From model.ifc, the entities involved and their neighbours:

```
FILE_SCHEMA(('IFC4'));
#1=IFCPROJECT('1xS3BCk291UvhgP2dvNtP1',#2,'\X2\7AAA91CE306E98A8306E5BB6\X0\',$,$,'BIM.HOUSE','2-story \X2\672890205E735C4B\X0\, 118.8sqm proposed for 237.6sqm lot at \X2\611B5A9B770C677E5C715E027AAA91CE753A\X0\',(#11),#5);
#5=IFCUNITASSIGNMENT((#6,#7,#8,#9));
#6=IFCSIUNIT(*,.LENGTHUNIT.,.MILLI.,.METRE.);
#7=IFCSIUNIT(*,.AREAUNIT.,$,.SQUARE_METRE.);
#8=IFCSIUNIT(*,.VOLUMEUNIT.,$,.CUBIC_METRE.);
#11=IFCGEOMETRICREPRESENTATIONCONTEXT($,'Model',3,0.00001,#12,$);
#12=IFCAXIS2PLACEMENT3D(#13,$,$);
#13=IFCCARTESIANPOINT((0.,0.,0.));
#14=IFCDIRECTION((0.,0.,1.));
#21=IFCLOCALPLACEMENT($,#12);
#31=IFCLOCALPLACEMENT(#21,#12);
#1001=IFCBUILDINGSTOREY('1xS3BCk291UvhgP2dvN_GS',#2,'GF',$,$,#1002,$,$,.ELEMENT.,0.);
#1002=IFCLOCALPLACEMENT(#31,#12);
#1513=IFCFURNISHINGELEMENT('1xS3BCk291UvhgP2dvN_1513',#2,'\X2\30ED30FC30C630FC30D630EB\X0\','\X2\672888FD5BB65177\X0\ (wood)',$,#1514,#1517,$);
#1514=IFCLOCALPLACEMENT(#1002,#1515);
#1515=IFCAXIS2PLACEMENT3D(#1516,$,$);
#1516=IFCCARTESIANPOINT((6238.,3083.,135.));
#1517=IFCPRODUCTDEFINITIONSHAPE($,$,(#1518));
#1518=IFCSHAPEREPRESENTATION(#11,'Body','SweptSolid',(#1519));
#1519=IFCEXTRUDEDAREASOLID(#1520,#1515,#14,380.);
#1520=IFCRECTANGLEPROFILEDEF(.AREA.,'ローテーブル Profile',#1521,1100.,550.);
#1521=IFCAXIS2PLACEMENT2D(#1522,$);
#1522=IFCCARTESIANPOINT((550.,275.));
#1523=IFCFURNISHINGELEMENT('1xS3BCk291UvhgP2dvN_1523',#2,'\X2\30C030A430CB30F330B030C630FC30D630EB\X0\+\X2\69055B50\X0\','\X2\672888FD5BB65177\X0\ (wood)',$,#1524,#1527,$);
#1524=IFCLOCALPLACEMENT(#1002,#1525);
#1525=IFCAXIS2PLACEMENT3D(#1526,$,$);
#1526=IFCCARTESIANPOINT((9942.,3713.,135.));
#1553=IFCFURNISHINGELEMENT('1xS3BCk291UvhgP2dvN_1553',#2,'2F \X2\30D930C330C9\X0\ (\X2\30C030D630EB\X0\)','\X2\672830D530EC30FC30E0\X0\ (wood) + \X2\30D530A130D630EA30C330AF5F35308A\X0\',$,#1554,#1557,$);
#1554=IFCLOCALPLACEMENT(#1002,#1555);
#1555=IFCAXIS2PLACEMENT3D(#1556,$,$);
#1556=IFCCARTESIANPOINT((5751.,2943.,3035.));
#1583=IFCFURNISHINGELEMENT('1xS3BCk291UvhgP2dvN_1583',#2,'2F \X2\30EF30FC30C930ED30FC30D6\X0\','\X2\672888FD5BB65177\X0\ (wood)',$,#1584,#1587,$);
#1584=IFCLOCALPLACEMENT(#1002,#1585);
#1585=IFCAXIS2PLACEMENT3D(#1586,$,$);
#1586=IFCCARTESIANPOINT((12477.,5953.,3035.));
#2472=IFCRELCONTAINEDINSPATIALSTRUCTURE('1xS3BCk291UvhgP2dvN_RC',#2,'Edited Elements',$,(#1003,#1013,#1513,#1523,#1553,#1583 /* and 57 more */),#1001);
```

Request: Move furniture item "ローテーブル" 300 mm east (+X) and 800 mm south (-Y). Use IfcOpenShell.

```python
import ifcopenshell
import ifcopenshell.api.geometry
import ifcopenshell.util.placement

model = ifcopenshell.open("model.ifc")

item = model.by_guid("1xS3BCk291UvhgP2dvN_1513")
matrix = ifcopenshell.util.placement.get_local_placement(item.ObjectPlacement)
matrix[0, 3] += 300.0
matrix[1, 3] -= 800.0
ifcopenshell.api.geometry.edit_object_placement(model, product=item, matrix=matrix, is_si=False)

print(ifcopenshell.util.placement.get_local_placement(item.ObjectPlacement).round(3) + 0.0)

model.write("model_v2.ifc")
```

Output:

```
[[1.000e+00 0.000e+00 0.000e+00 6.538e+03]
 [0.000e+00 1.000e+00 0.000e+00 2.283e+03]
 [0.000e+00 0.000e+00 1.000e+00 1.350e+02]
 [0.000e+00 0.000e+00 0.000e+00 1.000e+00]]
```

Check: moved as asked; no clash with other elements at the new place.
